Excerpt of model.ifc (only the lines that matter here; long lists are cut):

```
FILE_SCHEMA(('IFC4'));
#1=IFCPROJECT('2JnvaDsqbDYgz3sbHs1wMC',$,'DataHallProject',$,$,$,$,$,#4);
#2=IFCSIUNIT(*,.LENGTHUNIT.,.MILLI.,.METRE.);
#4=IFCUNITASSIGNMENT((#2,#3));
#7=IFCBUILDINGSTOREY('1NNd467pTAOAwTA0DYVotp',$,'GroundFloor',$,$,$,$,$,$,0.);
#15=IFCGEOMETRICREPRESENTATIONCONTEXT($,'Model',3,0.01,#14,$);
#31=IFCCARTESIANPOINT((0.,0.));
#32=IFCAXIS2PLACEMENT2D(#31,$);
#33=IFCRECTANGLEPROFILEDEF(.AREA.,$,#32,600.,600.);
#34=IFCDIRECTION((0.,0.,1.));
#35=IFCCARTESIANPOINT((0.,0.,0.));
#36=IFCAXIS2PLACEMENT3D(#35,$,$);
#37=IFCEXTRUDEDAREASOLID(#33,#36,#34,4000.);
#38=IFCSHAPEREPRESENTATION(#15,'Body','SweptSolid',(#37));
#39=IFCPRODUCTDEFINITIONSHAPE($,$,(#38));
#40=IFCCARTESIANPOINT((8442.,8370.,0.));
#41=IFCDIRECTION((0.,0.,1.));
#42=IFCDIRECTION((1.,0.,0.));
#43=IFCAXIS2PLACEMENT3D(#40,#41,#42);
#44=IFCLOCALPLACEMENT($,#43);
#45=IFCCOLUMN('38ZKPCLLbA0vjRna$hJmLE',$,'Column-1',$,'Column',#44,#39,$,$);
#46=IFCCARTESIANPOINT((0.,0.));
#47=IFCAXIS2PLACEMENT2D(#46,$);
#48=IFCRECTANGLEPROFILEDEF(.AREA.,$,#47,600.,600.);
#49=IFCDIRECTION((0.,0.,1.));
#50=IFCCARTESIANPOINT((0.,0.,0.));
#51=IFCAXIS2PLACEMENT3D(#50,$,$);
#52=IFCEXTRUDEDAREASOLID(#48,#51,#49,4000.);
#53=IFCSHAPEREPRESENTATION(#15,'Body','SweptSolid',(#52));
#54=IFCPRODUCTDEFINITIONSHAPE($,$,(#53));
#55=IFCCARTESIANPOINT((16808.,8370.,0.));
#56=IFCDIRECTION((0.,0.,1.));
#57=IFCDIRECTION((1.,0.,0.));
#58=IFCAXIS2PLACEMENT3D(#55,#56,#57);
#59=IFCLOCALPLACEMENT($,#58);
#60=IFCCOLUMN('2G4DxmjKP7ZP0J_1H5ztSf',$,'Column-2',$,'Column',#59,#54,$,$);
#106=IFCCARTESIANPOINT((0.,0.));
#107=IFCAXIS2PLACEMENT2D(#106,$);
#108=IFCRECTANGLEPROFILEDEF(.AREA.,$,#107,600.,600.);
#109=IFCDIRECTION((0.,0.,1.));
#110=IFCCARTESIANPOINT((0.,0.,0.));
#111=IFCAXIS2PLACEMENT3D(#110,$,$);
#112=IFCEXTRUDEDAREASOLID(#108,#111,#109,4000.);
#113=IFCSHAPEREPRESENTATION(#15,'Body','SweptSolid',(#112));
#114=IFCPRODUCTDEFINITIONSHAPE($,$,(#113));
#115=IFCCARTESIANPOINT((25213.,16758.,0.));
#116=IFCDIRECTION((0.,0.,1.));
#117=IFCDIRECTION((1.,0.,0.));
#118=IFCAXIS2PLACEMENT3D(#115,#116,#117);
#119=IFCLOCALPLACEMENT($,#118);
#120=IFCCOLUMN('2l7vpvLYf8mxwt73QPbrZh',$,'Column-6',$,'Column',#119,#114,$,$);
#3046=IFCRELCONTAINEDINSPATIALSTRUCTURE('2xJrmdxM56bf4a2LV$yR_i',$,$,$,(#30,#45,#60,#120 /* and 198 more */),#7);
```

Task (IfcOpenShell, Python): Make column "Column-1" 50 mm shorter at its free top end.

```python
import ifcopenshell

model = ifcopenshell.open("model.ifc")

member = model.by_guid("38ZKPCLLbA0vjRna$hJmLE")
change = -50.0

# The extrusion runs towards the end named, so only its depth changes.
body = next(r for r in member.Representation.Representations if r.RepresentationIdentifier == "Body")
solid = body.Items[0]
old_length = solid.Depth
solid.Depth += change

print(f"length {old_length:g} -> {solid.Depth:g}")

model.write("model_updated.ifc")
```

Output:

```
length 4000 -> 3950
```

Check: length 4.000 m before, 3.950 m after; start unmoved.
